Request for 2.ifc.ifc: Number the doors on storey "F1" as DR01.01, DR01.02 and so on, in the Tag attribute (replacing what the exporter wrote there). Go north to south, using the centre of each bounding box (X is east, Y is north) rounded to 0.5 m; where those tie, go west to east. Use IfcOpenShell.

First a look at what the model holds.

```python
import ifcopenshell
import ifcopenshell.util.element
import ifcopenshell.util.placement

model = ifcopenshell.open("2.ifc.ifc")
print(model.schema)
storey = next(s for s in model.by_type("IfcBuildingStorey") if s.Name == "F1")
doors = [e for e in ifcopenshell.util.element.get_decomposition(storey) if e.is_a("IfcDoor")]
for e in sorted(doors, key=lambda e: e.id()):
    origin = ifcopenshell.util.placement.get_local_placement(e.ObjectPlacement)[:3, 3]
    print(e.id(), e.Tag, e.Name, origin.round(2) + 0.0, sep=" | ")
```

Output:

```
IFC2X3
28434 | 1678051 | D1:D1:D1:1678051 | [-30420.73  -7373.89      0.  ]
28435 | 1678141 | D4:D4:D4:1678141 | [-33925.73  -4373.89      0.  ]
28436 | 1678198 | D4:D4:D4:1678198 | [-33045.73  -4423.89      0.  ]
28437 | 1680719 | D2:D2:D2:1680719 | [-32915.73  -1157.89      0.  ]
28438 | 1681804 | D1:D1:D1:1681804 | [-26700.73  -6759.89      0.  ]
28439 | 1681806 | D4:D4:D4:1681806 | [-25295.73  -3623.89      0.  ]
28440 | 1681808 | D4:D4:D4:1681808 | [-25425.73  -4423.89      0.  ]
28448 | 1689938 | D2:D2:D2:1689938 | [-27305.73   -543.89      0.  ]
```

```python
import ifcopenshell
import ifcopenshell.geom
import ifcopenshell.util.element
import ifcopenshell.util.shape

model = ifcopenshell.open("2.ifc.ifc")
settings = ifcopenshell.geom.settings()
settings.set("use-world-coords", True)


def centre(element):
    shape = ifcopenshell.geom.create_shape(settings, element)
    return ifcopenshell.util.shape.get_bbox_centroid(shape.geometry)


storey = next(s for s in model.by_type("IfcBuildingStorey") if s.Name == "F1")
doors = [e for e in ifcopenshell.util.element.get_decomposition(storey) if e.is_a("IfcDoor")]

# Insertion points can sit at a corner or the storey origin, so sort by the geometry (in metres).
centres = {e: centre(e) for e in doors}
doors.sort(key=lambda e: (-round(centres[e][1] / 0.5), centres[e][0]))

for i, e in enumerate(doors, start=1):
    number = f"DR01.{i:02d}"
    e.Tag = number
    print(e.id(), number)

model.write("2.ifc_updated.ifc")
```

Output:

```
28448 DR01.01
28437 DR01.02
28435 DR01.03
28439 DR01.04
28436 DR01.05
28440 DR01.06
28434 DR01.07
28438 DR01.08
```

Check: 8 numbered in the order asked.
